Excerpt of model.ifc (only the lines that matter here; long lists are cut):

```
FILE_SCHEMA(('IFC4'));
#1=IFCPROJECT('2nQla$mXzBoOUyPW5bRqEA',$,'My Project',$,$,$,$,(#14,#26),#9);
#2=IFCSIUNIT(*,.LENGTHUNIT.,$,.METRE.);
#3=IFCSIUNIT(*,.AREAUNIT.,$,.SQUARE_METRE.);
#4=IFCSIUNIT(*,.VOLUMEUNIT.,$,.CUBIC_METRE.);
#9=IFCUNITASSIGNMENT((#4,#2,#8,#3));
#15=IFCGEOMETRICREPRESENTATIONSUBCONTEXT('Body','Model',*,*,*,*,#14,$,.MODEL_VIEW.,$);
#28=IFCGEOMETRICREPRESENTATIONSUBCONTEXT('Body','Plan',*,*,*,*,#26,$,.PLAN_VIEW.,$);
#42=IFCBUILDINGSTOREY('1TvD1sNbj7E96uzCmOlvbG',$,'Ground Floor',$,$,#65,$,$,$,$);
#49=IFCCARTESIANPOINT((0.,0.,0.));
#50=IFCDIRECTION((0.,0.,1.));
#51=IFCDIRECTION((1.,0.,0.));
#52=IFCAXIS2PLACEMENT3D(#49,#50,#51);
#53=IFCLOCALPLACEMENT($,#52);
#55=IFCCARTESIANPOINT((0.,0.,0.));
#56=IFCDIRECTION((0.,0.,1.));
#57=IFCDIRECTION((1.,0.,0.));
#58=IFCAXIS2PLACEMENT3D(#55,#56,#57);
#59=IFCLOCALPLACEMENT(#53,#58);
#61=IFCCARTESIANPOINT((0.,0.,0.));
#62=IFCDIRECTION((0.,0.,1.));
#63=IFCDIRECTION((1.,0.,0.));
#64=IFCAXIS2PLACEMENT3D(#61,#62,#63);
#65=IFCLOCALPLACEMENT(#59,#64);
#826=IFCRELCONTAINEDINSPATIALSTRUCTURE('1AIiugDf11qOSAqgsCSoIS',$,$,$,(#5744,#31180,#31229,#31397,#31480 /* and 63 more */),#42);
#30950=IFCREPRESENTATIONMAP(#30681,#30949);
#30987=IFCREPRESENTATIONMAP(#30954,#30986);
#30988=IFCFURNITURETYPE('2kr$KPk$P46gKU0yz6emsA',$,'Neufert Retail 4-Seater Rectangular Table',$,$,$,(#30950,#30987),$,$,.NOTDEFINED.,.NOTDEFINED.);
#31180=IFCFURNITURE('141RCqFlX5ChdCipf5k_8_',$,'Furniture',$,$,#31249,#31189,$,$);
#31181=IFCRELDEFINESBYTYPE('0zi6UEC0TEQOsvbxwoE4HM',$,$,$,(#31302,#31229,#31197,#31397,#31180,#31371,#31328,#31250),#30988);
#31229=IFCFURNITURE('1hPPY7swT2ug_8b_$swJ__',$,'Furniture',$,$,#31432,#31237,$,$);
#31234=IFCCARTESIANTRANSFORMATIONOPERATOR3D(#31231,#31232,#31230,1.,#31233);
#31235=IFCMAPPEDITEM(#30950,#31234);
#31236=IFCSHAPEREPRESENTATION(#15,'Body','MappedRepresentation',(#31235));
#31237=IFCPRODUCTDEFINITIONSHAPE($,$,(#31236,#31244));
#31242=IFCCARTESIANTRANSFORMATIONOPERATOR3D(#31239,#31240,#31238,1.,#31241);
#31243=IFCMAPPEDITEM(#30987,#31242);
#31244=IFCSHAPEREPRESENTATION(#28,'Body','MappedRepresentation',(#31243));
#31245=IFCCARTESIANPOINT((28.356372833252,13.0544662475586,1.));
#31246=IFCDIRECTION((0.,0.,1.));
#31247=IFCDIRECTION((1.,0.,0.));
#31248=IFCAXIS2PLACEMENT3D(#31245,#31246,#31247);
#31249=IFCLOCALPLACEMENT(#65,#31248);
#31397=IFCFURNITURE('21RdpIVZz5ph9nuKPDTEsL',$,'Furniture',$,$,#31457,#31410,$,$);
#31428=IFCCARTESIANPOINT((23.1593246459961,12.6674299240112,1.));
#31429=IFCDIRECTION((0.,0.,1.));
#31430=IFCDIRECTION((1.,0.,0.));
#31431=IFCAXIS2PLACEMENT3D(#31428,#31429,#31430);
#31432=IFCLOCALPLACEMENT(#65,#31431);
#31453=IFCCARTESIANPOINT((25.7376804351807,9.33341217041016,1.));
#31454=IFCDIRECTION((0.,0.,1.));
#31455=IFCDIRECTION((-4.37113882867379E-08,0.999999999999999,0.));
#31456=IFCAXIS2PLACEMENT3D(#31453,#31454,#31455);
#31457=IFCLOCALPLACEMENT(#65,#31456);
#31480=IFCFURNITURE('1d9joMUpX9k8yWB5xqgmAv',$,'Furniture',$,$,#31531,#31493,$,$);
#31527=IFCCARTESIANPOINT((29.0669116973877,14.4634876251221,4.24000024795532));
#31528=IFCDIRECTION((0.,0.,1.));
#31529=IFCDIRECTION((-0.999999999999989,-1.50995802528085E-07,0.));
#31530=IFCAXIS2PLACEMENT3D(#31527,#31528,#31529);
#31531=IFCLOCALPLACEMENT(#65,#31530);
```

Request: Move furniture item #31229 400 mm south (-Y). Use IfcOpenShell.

```python
import ifcopenshell
import ifcopenshell.api.geometry
import ifcopenshell.util.placement
import ifcopenshell.util.unit

model = ifcopenshell.open("model.ifc")
unit_scale = ifcopenshell.util.unit.calculate_unit_scale(model)

item = model.by_guid("1hPPY7swT2ug_8b_$swJ__")
matrix = ifcopenshell.util.placement.get_local_placement(item.ObjectPlacement)
matrix[1, 3] -= 0.4 / unit_scale
ifcopenshell.api.geometry.edit_object_placement(model, product=item, matrix=matrix, is_si=False)

print(ifcopenshell.util.placement.get_local_placement(item.ObjectPlacement).round(3) + 0.0)

model.write("model_updated.ifc")
```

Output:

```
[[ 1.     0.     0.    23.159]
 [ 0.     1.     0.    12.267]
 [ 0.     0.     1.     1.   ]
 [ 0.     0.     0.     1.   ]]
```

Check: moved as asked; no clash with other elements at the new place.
